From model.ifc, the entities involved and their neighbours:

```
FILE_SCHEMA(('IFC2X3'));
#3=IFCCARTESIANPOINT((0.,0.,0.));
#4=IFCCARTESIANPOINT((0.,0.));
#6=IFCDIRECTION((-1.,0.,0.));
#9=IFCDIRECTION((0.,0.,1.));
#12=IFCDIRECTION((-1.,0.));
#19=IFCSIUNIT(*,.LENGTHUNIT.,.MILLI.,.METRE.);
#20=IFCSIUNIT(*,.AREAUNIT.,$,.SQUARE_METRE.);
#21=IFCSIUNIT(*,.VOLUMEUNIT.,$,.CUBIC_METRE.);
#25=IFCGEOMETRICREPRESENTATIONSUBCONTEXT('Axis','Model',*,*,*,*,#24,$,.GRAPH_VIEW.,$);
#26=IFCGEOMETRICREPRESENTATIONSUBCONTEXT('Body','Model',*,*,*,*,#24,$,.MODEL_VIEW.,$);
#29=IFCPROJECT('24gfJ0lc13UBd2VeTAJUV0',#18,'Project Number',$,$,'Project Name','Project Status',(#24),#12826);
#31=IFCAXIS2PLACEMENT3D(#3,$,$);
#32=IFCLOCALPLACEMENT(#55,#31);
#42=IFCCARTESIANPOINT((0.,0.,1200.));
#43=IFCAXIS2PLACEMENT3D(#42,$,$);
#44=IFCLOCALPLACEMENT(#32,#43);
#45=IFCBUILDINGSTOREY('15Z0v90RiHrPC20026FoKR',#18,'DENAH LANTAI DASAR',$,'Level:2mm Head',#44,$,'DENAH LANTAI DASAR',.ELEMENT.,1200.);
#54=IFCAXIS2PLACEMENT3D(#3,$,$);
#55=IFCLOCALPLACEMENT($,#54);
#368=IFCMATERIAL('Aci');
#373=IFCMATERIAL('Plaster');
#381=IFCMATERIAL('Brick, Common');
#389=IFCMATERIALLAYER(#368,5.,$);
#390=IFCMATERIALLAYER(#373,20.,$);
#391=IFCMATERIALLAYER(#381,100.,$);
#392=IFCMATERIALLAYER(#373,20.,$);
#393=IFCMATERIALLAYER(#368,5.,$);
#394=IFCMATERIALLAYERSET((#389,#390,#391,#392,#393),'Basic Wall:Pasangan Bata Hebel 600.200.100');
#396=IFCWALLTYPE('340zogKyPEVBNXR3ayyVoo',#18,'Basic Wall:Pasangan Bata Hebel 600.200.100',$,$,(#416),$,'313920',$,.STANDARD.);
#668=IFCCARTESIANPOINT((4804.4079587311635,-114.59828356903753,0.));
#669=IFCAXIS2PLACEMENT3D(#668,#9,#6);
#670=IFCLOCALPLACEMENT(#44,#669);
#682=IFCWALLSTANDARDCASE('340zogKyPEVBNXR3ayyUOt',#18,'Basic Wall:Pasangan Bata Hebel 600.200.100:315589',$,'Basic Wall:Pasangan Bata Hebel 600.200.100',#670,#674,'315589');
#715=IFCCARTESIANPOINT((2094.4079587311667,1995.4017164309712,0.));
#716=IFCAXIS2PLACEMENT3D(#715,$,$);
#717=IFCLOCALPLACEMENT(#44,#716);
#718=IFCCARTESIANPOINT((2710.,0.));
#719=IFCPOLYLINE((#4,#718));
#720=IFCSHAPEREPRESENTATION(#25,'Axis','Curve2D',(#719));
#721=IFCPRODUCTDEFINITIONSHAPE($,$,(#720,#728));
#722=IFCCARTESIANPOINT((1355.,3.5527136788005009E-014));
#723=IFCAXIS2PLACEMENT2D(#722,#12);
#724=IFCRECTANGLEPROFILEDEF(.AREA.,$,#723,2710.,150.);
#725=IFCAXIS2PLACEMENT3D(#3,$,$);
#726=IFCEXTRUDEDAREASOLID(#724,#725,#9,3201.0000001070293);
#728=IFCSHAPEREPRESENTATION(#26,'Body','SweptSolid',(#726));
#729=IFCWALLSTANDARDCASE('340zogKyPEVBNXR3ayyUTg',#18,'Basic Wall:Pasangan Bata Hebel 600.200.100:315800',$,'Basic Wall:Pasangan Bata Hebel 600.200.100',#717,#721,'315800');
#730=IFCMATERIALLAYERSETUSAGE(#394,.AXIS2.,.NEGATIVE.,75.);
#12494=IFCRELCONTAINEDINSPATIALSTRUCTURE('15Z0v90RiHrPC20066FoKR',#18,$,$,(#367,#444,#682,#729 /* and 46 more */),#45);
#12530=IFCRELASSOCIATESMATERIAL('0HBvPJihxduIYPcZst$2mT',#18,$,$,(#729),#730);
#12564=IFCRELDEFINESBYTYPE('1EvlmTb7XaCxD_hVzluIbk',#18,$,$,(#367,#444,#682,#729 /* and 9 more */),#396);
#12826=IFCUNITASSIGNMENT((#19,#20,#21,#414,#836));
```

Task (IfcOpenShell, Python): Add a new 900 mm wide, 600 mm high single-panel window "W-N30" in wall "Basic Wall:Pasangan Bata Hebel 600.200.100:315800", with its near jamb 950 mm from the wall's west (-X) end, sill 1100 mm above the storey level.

```python
import numpy as np
import ifcopenshell
import ifcopenshell.api.feature
import ifcopenshell.api.geometry
import ifcopenshell.api.root
import ifcopenshell.api.spatial
import ifcopenshell.api.type
import ifcopenshell.geom
import ifcopenshell.util.element
import ifcopenshell.util.placement
import ifcopenshell.util.representation
import ifcopenshell.util.shape
import ifcopenshell.util.unit

model = ifcopenshell.open("model.ifc")
unit_scale = ifcopenshell.util.unit.calculate_unit_scale(model)
settings = ifcopenshell.geom.settings()


def volume(element):
    """Net volume in cubic metres, openings subtracted."""
    shape = ifcopenshell.geom.create_shape(settings, element)
    return ifcopenshell.util.shape.get_volume(shape.geometry)


wall = model.by_guid("340zogKyPEVBNXR3ayyUTg")
storey = ifcopenshell.util.element.get_container(wall, ifc_class="IfcBuildingStorey")
context = ifcopenshell.util.representation.get_context(model, "Model", "Body", "MODEL_VIEW")
before = volume(wall)

width, height, from_end, sill = 0.9, 0.6, 0.95, 1.1  # metres

# The wall runs along its own X axis, and the end named is its -X end.
wall_shape = ifcopenshell.geom.create_shape(settings, wall)
x, y, z = ifcopenshell.util.shape.get_vertices(wall_shape.geometry).T
start = x.min() + from_end
face, thickness = float(y.min()), float(y.max() - y.min())
wall_matrix = ifcopenshell.util.placement.get_local_placement(wall.ObjectPlacement)
level = ifcopenshell.util.placement.get_local_placement(storey.ObjectPlacement)[2, 3]


def in_wall(x, y):
    """Placement at x, y metres in the wall's axes, at sill height."""
    matrix = wall_matrix.copy()
    matrix[:, 3] = wall_matrix @ np.array([x / unit_scale, y / unit_scale, 0.0, 1.0])
    matrix[2, 3] = level + sill / unit_scale
    return matrix


# Opening: a box that overshoots both wall faces by 50 mm.
opening = ifcopenshell.api.root.create_entity(model, ifc_class="IfcOpeningElement")
box = ifcopenshell.api.geometry.add_wall_representation(
    model, context=context, length=width, height=height, thickness=thickness + 0.1
)
ifcopenshell.api.geometry.assign_representation(model, product=opening, representation=box)
ifcopenshell.api.geometry.edit_object_placement(model, product=opening, matrix=in_wall(start, face - 0.05), is_si=False)
ifcopenshell.api.feature.add_feature(model, feature=opening, element=wall)

window = ifcopenshell.api.root.create_entity(model, ifc_class="IfcWindow", name="W-N30")
window.OverallWidth, window.OverallHeight = width / unit_scale, height / unit_scale
body = ifcopenshell.api.geometry.add_window_representation(
    model,
    context=context,
    overall_width=window.OverallWidth,
    overall_height=window.OverallHeight,
    partition_type="SINGLE_PANEL",
)
ifcopenshell.api.geometry.assign_representation(model, product=window, representation=body)
ifcopenshell.api.spatial.assign_container(model, products=[window], relating_structure=storey)
fills = ifcopenshell.api.feature.add_filling(model, opening=opening, element=window)
fills.OwnerHistory = window.OwnerHistory  # required in IFC2X3

# IFC2X3 keeps the operation on the window style.
style = ifcopenshell.api.root.create_entity(model, ifc_class="IfcWindowStyle", name="W-N30")
style.OperationType, style.ConstructionType = "SINGLE_PANEL", "NOTDEFINED"
style.ParameterTakesPrecedence = style.Sizeable = False
ifcopenshell.api.type.assign_type(model, related_objects=[window], relating_type=style)

# Centre the window in the wall's thickness.
ifcopenshell.api.geometry.edit_object_placement(model, product=window, matrix=in_wall(start, face), is_si=False)
window_shape = ifcopenshell.geom.create_shape(settings, window)
depth = ifcopenshell.util.shape.get_vertices(window_shape.geometry)[:, 1]
offset = face + thickness / 2 - (depth.min() + depth.max()) / 2
ifcopenshell.api.geometry.edit_object_placement(model, product=window, matrix=in_wall(start, offset), is_si=False)

after = volume(wall)

print(f"wall volume {before:.3f} -> {after:.3f} m3")

model.write("model-out.ifc")
```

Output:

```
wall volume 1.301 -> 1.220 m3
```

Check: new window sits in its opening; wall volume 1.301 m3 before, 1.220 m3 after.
